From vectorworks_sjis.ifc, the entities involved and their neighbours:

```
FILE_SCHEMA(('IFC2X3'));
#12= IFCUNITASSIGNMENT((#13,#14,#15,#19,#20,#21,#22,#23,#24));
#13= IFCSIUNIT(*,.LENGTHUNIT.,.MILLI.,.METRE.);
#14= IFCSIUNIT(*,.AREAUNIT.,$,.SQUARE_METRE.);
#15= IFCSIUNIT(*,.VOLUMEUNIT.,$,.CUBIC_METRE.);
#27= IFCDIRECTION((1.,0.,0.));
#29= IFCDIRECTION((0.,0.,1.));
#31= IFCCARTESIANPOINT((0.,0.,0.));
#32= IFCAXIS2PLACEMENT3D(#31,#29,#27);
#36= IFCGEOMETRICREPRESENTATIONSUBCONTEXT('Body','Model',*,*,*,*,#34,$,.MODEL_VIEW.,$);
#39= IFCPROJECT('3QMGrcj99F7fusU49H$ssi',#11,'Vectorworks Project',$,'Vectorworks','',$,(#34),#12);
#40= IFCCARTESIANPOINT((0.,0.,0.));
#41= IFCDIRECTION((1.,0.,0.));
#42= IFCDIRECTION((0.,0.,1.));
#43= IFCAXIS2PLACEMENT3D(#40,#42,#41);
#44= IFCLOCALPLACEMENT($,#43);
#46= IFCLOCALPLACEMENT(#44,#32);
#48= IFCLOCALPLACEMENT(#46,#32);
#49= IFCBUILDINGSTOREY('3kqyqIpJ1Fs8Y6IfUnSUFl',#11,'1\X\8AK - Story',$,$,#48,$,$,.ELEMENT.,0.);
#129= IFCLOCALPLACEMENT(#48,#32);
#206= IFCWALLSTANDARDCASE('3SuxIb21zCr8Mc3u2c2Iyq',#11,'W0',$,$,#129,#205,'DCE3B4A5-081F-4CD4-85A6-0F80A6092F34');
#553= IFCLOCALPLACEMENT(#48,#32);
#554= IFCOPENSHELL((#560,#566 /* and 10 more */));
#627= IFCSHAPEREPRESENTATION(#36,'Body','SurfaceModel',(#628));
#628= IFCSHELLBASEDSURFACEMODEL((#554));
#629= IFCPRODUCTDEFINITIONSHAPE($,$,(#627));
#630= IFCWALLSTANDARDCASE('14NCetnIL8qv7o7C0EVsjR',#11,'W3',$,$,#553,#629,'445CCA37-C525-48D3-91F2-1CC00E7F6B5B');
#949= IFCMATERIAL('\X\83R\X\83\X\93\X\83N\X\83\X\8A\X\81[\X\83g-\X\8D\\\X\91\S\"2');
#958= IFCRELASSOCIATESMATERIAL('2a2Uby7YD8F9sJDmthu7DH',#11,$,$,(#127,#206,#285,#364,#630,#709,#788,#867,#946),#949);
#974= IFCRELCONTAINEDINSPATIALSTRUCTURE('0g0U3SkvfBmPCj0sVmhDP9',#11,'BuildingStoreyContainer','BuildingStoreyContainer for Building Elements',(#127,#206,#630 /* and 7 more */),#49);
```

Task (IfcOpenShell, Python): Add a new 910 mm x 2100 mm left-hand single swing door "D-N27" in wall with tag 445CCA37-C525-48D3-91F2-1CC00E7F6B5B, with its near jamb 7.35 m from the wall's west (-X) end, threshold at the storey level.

```python
import numpy as np
import ifcopenshell
import ifcopenshell.api.feature
import ifcopenshell.api.geometry
import ifcopenshell.api.root
import ifcopenshell.api.spatial
import ifcopenshell.api.type
import ifcopenshell.geom
import ifcopenshell.util.element
import ifcopenshell.util.placement
import ifcopenshell.util.representation
import ifcopenshell.util.shape
import ifcopenshell.util.unit

model = ifcopenshell.open("vectorworks_sjis.ifc")
unit_scale = ifcopenshell.util.unit.calculate_unit_scale(model)
settings = ifcopenshell.geom.settings()


def volume(element):
    """Net volume in cubic metres, openings subtracted."""
    shape = ifcopenshell.geom.create_shape(settings, element)
    return ifcopenshell.util.shape.get_volume(shape.geometry)


wall = model.by_id(630)
storey = ifcopenshell.util.element.get_container(wall, ifc_class="IfcBuildingStorey")
context = ifcopenshell.util.representation.get_context(model, "Model", "Body", "MODEL_VIEW")
before = volume(wall)

width, height, from_end, sill = 0.91, 2.1, 7.35, 0.0  # metres

# The wall runs along its own X axis, and the end named is its -X end.
wall_shape = ifcopenshell.geom.create_shape(settings, wall)
x, y, z = ifcopenshell.util.shape.get_vertices(wall_shape.geometry).T
start = x.min() + from_end
face, thickness = float(y.min()), float(y.max() - y.min())
wall_matrix = ifcopenshell.util.placement.get_local_placement(wall.ObjectPlacement)
level = ifcopenshell.util.placement.get_local_placement(storey.ObjectPlacement)[2, 3]


def in_wall(x, y):
    """Placement at x, y metres in the wall's axes, at sill height."""
    matrix = wall_matrix.copy()
    matrix[:, 3] = wall_matrix @ np.array([x / unit_scale, y / unit_scale, 0.0, 1.0])
    matrix[2, 3] = level + sill / unit_scale
    return matrix


# Opening: a box that overshoots both wall faces by 50 mm.
opening = ifcopenshell.api.root.create_entity(model, ifc_class="IfcOpeningElement")
box = ifcopenshell.api.geometry.add_wall_representation(
    model, context=context, length=width, height=height, thickness=thickness + 0.1
)
ifcopenshell.api.geometry.assign_representation(model, product=opening, representation=box)
ifcopenshell.api.geometry.edit_object_placement(model, product=opening, matrix=in_wall(start, face - 0.05), is_si=False)
ifcopenshell.api.feature.add_feature(model, feature=opening, element=wall)

door = ifcopenshell.api.root.create_entity(model, ifc_class="IfcDoor", name="D-N27")
door.OverallWidth, door.OverallHeight = width / unit_scale, height / unit_scale
body = ifcopenshell.api.geometry.add_door_representation(
    model,
    context=context,
    overall_width=door.OverallWidth,
    overall_height=door.OverallHeight,
    operation_type="SINGLE_SWING_LEFT",
    lining_properties={"LiningDepth": thickness / unit_scale, "ThresholdDepth": thickness / unit_scale},
)
ifcopenshell.api.geometry.assign_representation(model, product=door, representation=body)
ifcopenshell.api.spatial.assign_container(model, products=[door], relating_structure=storey)
fills = ifcopenshell.api.feature.add_filling(model, opening=opening, element=door)
fills.OwnerHistory = door.OwnerHistory  # required in IFC2X3

# IFC2X3 keeps the operation on the door style.
style = ifcopenshell.api.root.create_entity(model, ifc_class="IfcDoorStyle", name="D-N27")
style.OperationType, style.ConstructionType = "SINGLE_SWING_LEFT", "NOTDEFINED"
style.ParameterTakesPrecedence = style.Sizeable = False
ifcopenshell.api.type.assign_type(model, related_objects=[door], relating_type=style)

# The lining spans the wall, so the door starts at the wall face.
ifcopenshell.api.geometry.edit_object_placement(model, product=door, matrix=in_wall(start, face), is_si=False)

after = volume(wall)

print(f"wall volume {before:.3f} -> {after:.3f} m3")

model.write("vectorworks_sjis_v2.ifc")
```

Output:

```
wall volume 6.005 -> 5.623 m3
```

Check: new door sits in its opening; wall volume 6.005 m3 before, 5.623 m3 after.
